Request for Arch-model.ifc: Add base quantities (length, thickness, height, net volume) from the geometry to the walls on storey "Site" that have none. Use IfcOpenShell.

First a look at what the model holds.

```python
import ifcopenshell
import ifcopenshell.util.element
import ifcopenshell.util.unit

model = ifcopenshell.open("Arch-model.ifc")
print(model.schema)
for unit_type in ("LENGTHUNIT", "AREAUNIT", "VOLUMEUNIT"):
    print(unit_type, ifcopenshell.util.unit.calculate_unit_scale(model, unit_type))
storey = next(s for s in model.by_type("IfcBuildingStorey") if s.Name == "Site")
walls = [e for e in ifcopenshell.util.element.get_decomposition(storey) if e.is_a("IfcWall")]
for e in sorted(walls, key=lambda e: e.id()):
    print(e.id(), e.is_a(), e.Name, list(ifcopenshell.util.element.get_psets(e, qtos_only=True)), sep=" | ")
```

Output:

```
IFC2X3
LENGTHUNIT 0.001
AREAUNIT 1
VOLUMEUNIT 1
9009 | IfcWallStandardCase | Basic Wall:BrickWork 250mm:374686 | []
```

```python
import ifcopenshell
import ifcopenshell.api.pset
import ifcopenshell.geom
import ifcopenshell.util.element
import ifcopenshell.util.shape
import ifcopenshell.util.unit

model = ifcopenshell.open("Arch-model.ifc")
unit_scale = ifcopenshell.util.unit.calculate_unit_scale(model)
volume_scale = ifcopenshell.util.unit.calculate_unit_scale(model, "VOLUMEUNIT")
settings = ifcopenshell.geom.settings()

storey = next(s for s in model.by_type("IfcBuildingStorey") if s.Name == "Site")
walls = [e for e in ifcopenshell.util.element.get_decomposition(storey) if e.is_a("IfcWall")]

for e in sorted(walls, key=lambda e: e.id()):
    if ifcopenshell.util.element.get_psets(e, qtos_only=True, should_inherit=False):
        continue
    # Geometry comes back in metres, in the element's own axes.
    shape = ifcopenshell.geom.create_shape(settings, e)
    values = {
        "Length": ifcopenshell.util.shape.get_x(shape.geometry) / unit_scale,
        "Width": ifcopenshell.util.shape.get_y(shape.geometry) / unit_scale,
        "Height": ifcopenshell.util.shape.get_z(shape.geometry) / unit_scale,
        "NetVolume": ifcopenshell.util.shape.get_volume(shape.geometry) / volume_scale,
    }
    qto = ifcopenshell.api.pset.add_qto(model, product=e, name="BaseQuantities")
    ifcopenshell.api.pset.edit_qto(model, qto=qto, properties=values)
    print(e.id(), {k: round(v, 3) for k, v in values.items()})

model.write("Arch-model_v2.ifc")
```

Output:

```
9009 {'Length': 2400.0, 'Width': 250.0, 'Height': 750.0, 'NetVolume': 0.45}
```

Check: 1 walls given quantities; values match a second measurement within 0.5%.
